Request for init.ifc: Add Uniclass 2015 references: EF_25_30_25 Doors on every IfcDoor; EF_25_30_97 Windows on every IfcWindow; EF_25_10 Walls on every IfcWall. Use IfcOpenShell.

First a look at what the model holds.

```python
import ifcopenshell

model = ifcopenshell.open("init.ifc")
print(model.schema)
print("classifications:", [c.Name for c in model.by_type("IfcClassification")])
for ifc_class in ("IfcDoor", "IfcRoof", "IfcStair", "IfcWall", "IfcWindow"):
    print(ifc_class, len(model.by_type(ifc_class)))
```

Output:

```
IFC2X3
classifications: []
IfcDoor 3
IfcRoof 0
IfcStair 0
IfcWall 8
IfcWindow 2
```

```python
import ifcopenshell
import ifcopenshell.api.classification

model = ifcopenshell.open("init.ifc")

# IFC2X3 requires Source and Edition and has no link from the project to the system.
system = model.create_entity("IfcClassification", Source="NBS", Edition="2015", Name="Uniclass 2015")

codes = {
    "IfcDoor": ("EF_25_30_25", "Doors"),
    "IfcWindow": ("EF_25_30_97", "Windows"),
    "IfcWall": ("EF_25_10", "Walls"),
}
for ifc_class, (code, name) in codes.items():
    products = model.by_type(ifc_class)
    ifcopenshell.api.classification.add_reference(
        model, products=products, classification=system, identification=code, name=name
    )
    print(code, len(products))

model.write("init_updated.ifc")
```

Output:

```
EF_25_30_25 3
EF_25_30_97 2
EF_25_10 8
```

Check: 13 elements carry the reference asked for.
